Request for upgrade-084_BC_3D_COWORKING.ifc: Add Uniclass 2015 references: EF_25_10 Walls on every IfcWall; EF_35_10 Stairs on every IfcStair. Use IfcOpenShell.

First a look at what the model holds.

```python
import ifcopenshell

model = ifcopenshell.open("upgrade-084_BC_3D_COWORKING.ifc")
print(model.schema)
print("classifications:", [c.Name for c in model.by_type("IfcClassification")])
for ifc_class in ("IfcDoor", "IfcRoof", "IfcStair", "IfcWall", "IfcWindow"):
    print(ifc_class, len(model.by_type(ifc_class)))
```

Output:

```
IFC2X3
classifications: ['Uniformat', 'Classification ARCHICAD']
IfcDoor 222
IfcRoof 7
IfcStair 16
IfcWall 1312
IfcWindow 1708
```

```python
import ifcopenshell
import ifcopenshell.api.classification

model = ifcopenshell.open("upgrade-084_BC_3D_COWORKING.ifc")

# IFC2X3 requires Source and Edition and has no link from the project to the system.
system = model.create_entity("IfcClassification", Source="NBS", Edition="2015", Name="Uniclass 2015")

codes = {
    "IfcWall": ("EF_25_10", "Walls"),
    "IfcStair": ("EF_35_10", "Stairs"),
}
for ifc_class, (code, name) in codes.items():
    products = model.by_type(ifc_class)
    ifcopenshell.api.classification.add_reference(
        model, products=products, classification=system, identification=code, name=name
    )
    print(code, len(products))

model.write("upgrade-084_BC_3D_COWORKING_edited.ifc")
```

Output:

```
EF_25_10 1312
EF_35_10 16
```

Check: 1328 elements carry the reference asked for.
